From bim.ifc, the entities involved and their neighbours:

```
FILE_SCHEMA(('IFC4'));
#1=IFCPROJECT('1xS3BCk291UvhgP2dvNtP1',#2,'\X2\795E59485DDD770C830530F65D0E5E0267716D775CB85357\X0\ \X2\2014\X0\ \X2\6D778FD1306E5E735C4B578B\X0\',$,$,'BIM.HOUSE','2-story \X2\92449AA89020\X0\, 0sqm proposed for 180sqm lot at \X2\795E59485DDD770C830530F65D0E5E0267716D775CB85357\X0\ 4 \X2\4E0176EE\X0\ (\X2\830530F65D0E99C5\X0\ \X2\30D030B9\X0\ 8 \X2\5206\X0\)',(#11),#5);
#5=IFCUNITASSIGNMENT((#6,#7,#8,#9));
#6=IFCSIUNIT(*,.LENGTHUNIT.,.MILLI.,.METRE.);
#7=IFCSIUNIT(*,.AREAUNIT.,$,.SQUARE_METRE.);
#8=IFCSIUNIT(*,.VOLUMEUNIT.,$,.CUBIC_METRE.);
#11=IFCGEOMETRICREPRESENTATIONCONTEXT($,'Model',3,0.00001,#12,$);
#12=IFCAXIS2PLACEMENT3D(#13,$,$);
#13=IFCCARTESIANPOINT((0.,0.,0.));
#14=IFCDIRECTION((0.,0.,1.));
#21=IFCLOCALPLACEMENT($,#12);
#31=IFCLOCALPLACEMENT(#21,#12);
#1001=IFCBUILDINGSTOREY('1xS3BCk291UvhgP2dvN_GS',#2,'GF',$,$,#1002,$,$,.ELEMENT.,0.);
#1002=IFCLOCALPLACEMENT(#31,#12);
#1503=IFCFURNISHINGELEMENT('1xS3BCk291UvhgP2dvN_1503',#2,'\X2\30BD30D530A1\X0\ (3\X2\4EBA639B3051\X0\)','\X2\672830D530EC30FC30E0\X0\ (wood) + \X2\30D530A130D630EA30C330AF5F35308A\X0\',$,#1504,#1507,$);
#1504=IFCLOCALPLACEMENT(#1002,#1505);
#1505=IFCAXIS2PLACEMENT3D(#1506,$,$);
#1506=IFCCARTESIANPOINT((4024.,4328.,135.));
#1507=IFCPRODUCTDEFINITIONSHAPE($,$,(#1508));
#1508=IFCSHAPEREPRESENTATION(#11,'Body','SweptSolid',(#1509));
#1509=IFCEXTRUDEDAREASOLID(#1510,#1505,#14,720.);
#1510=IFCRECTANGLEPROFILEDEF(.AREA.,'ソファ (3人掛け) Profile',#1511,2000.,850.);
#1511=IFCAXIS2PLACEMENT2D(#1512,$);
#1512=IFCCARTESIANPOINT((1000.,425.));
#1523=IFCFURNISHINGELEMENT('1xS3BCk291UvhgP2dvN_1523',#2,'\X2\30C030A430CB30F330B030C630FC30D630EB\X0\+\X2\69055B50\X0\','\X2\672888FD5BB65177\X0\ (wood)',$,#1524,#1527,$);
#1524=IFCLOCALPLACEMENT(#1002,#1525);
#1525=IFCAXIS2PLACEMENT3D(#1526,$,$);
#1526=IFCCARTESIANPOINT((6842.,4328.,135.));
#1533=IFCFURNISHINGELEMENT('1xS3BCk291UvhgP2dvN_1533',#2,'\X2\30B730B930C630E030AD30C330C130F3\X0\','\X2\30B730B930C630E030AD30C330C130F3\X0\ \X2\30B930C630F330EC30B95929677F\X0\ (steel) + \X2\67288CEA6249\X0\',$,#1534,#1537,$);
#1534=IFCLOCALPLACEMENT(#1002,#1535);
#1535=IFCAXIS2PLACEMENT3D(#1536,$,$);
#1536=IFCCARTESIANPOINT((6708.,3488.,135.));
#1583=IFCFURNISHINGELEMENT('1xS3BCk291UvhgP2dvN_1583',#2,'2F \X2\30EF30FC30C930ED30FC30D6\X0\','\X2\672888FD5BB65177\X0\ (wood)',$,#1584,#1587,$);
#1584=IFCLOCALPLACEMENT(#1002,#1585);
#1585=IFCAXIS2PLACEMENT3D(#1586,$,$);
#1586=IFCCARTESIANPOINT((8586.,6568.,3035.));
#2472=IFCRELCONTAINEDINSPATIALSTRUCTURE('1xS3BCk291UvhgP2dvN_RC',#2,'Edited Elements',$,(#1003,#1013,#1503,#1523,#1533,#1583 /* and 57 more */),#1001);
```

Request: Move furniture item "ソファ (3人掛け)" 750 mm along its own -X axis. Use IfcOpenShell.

```python
import ifcopenshell
import ifcopenshell.api.geometry
import ifcopenshell.util.placement
import ifcopenshell.util.unit

model = ifcopenshell.open("bim.ifc")
unit_scale = ifcopenshell.util.unit.calculate_unit_scale(model)

item = model.by_guid("1xS3BCk291UvhgP2dvN_1503")
matrix = ifcopenshell.util.placement.get_local_placement(item.ObjectPlacement)
matrix[:3, 3] -= matrix[:3, 0] * 0.75 / unit_scale
ifcopenshell.api.geometry.edit_object_placement(model, product=item, matrix=matrix, is_si=False)

print(ifcopenshell.util.placement.get_local_placement(item.ObjectPlacement).round(3) + 0.0)

model.write("bim_updated.ifc")
```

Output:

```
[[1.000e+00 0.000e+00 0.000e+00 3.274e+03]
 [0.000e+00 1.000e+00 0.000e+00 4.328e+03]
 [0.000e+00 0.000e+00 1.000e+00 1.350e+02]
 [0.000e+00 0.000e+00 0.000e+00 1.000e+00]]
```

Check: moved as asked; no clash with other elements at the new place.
